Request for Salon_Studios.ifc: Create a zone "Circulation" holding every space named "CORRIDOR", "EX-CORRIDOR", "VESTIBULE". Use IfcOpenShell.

First a look at what the model holds.

```python
import ifcopenshell

model = ifcopenshell.open("Salon_Studios.ifc")
print(model.schema)
seen = {}
for space in model.by_type("IfcSpace"):
    seen[space.LongName] = seen.get(space.LongName, 0) + 1
for name, count in sorted(seen.items(), key=str):
    print(count, "x", name)
print("zones:", [z.Name for z in model.by_type("IfcZone")][:20])
```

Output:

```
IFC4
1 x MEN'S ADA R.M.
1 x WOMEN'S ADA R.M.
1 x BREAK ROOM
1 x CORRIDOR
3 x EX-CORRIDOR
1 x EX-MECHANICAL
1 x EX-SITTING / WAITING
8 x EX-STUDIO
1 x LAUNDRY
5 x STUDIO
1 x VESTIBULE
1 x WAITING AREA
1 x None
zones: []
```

```python
import ifcopenshell
import ifcopenshell.api.group
import ifcopenshell.api.root

model = ifcopenshell.open("Salon_Studios.ifc")

names = {"CORRIDOR", "EX-CORRIDOR", "VESTIBULE"}
spaces = [s for s in model.by_type("IfcSpace") if s.LongName in names]

zone = ifcopenshell.api.root.create_entity(model, ifc_class="IfcZone", name="Circulation")
ifcopenshell.api.group.assign_group(model, products=spaces, group=zone)
print(len(spaces), "spaces in", zone.Name)

model.write("Salon_Studios_v2.ifc")
```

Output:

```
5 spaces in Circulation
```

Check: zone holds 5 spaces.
